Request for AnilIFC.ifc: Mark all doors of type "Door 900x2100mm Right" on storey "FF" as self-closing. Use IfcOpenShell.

First a look at what the model holds.

```python
import ifcopenshell
import ifcopenshell.util.element

model = ifcopenshell.open("AnilIFC.ifc")
print(model.schema)
storey = next(s for s in model.by_type("IfcBuildingStorey") if s.Name == "FF")
doors = [e for e in ifcopenshell.util.element.get_decomposition(storey) if e.is_a("IfcDoor")]
seen = {}
for e in doors:
    element_type = ifcopenshell.util.element.get_type(e)
    key = (element_type.Name if element_type != e and element_type else None, ifcopenshell.util.element.get_pset(e, "Pset_DoorCommon", "SelfClosing"))
    seen[key] = seen.get(key, 0) + 1
for (name, value), count in sorted(seen.items(), key=str):
    print(count, "x", name, "|", value)
```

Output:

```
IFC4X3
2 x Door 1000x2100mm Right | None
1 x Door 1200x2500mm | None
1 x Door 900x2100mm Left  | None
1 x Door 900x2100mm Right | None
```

```python
import ifcopenshell
import ifcopenshell.api.pset
import ifcopenshell.util.element

model = ifcopenshell.open("AnilIFC.ifc")

storey = next(s for s in model.by_type("IfcBuildingStorey") if s.Name == "FF")
doors = [e for e in ifcopenshell.util.element.get_decomposition(storey) if e.is_a("IfcDoor")]

count = 0
for e in doors:
    element_type = ifcopenshell.util.element.get_type(e)
    if element_type in (None, e) or element_type.Name != "Door 900x2100mm Right":
        continue
    # add_pset returns the element's existing set when there is one.
    pset = ifcopenshell.api.pset.add_pset(model, product=e, name="Pset_DoorCommon")
    ifcopenshell.api.pset.edit_pset(model, pset=pset, properties={"SelfClosing": True})
    count += 1

print(count, "doors updated")

model.write("AnilIFC_rev.ifc")
```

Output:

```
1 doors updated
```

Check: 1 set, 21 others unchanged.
